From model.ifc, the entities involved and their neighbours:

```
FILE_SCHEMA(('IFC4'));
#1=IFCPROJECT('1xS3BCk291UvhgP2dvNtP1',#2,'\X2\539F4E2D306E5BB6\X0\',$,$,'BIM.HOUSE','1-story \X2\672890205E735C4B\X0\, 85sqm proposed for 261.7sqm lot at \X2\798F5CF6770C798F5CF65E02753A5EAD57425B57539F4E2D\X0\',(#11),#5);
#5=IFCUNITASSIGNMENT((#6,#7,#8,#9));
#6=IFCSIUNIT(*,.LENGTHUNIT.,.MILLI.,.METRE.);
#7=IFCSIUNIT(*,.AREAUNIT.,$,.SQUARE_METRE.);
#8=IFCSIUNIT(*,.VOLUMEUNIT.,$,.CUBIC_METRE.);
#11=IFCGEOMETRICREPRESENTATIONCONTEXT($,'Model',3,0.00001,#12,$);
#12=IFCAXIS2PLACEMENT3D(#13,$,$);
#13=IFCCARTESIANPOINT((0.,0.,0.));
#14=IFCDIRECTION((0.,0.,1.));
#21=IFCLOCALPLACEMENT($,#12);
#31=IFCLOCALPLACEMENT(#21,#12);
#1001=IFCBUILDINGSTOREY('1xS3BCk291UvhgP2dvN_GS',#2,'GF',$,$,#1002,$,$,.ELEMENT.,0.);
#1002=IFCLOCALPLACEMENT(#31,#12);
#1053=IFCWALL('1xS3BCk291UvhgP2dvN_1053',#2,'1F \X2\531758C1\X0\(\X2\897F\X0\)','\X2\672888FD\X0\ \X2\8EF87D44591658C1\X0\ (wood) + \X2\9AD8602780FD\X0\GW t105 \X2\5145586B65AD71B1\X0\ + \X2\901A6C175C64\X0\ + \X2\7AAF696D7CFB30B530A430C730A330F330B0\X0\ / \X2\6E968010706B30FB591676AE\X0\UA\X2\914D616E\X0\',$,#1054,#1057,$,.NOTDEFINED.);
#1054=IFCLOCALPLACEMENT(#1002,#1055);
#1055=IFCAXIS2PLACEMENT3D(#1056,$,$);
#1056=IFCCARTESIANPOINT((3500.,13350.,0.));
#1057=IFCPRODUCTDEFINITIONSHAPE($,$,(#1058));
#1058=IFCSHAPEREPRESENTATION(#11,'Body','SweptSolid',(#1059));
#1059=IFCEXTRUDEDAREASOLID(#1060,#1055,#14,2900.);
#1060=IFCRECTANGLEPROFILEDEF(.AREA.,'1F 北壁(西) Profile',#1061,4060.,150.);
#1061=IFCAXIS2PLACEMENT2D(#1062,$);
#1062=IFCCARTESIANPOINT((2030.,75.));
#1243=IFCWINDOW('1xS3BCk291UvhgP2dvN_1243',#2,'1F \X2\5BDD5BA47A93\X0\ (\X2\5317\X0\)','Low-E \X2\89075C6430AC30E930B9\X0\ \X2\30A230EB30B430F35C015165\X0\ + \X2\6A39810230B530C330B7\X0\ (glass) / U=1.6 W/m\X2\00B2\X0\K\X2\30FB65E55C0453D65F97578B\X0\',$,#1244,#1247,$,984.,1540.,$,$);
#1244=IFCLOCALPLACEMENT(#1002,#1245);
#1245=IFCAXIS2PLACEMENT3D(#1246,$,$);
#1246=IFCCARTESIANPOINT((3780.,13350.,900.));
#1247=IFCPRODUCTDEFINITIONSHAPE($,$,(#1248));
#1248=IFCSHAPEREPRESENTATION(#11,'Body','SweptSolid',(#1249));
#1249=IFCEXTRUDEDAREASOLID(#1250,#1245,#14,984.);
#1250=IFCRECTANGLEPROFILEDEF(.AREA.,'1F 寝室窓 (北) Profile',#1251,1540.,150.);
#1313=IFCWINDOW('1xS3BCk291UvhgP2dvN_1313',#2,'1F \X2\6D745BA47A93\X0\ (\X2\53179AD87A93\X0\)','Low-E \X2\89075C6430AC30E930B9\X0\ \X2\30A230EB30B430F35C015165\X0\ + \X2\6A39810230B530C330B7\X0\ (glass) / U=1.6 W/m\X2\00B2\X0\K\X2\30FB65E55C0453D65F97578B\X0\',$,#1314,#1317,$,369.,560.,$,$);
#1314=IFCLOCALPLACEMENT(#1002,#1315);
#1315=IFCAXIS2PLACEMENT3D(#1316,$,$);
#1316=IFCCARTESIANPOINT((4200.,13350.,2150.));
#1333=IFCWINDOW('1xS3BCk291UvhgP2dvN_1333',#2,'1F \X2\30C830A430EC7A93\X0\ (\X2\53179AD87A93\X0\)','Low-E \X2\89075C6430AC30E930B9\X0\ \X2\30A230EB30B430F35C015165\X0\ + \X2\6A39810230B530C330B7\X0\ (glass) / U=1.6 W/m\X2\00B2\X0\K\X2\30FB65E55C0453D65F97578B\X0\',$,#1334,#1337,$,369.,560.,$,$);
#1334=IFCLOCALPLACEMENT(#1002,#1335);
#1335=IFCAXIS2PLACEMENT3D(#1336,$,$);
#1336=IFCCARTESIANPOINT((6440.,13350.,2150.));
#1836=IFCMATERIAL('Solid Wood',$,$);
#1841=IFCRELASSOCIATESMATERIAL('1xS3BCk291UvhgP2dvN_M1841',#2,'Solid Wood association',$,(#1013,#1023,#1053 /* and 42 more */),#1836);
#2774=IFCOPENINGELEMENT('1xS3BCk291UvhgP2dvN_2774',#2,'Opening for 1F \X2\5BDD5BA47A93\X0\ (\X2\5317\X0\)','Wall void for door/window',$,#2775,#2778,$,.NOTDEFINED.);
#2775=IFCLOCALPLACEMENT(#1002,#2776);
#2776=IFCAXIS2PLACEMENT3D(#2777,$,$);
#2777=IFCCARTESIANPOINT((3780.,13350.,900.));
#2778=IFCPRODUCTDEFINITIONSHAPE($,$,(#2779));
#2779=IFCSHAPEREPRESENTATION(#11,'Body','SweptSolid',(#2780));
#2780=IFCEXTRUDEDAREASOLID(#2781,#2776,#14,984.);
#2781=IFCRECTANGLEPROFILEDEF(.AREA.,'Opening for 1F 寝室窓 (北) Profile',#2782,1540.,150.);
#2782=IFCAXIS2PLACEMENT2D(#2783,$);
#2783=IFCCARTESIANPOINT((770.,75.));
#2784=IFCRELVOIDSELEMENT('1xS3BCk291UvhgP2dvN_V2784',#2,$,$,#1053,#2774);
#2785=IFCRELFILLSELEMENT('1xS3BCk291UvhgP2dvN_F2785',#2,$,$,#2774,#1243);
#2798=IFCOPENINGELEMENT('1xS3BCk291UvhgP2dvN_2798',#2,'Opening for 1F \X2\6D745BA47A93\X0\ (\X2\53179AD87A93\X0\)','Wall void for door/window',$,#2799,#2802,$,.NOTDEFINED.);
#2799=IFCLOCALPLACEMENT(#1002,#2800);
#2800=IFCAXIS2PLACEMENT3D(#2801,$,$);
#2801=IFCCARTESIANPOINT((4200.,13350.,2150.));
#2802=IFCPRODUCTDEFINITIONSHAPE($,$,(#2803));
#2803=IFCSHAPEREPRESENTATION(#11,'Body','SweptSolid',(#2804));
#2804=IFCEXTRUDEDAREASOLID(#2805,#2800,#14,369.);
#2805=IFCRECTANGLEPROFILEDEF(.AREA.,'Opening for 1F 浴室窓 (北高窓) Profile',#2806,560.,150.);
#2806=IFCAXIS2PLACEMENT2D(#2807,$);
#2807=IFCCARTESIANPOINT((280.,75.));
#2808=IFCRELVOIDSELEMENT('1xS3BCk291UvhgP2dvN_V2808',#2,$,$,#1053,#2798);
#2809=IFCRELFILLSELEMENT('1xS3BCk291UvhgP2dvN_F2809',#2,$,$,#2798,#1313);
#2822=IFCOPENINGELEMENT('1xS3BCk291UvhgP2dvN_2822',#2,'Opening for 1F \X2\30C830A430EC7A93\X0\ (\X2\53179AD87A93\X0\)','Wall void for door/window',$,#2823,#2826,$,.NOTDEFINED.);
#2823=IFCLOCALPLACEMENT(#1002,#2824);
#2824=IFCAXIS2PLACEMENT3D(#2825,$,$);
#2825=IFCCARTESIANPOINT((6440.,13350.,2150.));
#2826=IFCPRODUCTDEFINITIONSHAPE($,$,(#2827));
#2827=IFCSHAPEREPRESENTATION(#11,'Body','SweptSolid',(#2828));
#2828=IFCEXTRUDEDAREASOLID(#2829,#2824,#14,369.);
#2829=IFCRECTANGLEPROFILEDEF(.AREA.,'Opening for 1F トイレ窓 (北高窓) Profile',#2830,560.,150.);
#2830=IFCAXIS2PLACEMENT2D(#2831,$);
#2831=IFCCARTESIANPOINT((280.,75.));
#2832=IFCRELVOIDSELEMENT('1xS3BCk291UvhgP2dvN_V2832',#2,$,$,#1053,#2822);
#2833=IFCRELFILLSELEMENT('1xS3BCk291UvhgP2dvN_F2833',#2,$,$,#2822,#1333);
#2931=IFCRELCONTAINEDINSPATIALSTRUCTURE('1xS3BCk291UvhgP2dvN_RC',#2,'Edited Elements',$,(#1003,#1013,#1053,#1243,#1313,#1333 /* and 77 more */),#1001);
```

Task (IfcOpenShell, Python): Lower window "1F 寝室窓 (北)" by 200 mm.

```python
import numpy as np
import ifcopenshell
import ifcopenshell.api.geometry
import ifcopenshell.util.placement
import ifcopenshell.util.unit

model = ifcopenshell.open("model.ifc")
unit_scale = ifcopenshell.util.unit.calculate_unit_scale(model)

window = model.by_guid("1xS3BCk291UvhgP2dvN_1243")
opening = window.FillsVoids[0].RelatingOpeningElement
dz = -200.0

shift = np.array([0.0, 0.0, dz])
# The window is not placed relative to its opening, so move both.
for product in (opening, window):
    matrix = ifcopenshell.util.placement.get_local_placement(product.ObjectPlacement)
    matrix[:3, 3] += shift
    ifcopenshell.api.geometry.edit_object_placement(model, product=product, matrix=matrix, is_si=False)

print(f"moved by {dz * unit_scale:+.3f} m")

model.write("model_edited.ifc")
```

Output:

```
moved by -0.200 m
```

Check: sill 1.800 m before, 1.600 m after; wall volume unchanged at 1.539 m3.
